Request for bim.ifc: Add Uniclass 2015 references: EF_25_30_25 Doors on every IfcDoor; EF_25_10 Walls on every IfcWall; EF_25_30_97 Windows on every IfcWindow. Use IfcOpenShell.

First a look at what the model holds.

```python
import ifcopenshell

model = ifcopenshell.open("bim.ifc")
print(model.schema)
print("classifications:", [c.Name for c in model.by_type("IfcClassification")])
for ifc_class in ("IfcDoor", "IfcRoof", "IfcStair", "IfcWall", "IfcWindow"):
    print(ifc_class, len(model.by_type(ifc_class)))
```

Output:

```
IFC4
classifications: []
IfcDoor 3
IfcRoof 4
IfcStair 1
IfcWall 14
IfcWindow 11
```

```python
import ifcopenshell
import ifcopenshell.api.classification

model = ifcopenshell.open("bim.ifc")

system = ifcopenshell.api.classification.add_classification(model, classification="Uniclass 2015")

codes = {
    "IfcDoor": ("EF_25_30_25", "Doors"),
    "IfcWall": ("EF_25_10", "Walls"),
    "IfcWindow": ("EF_25_30_97", "Windows"),
}
for ifc_class, (code, name) in codes.items():
    products = model.by_type(ifc_class)
    ifcopenshell.api.classification.add_reference(
        model, products=products, classification=system, identification=code, name=name
    )
    print(code, len(products))

model.write("bim_edited.ifc")
```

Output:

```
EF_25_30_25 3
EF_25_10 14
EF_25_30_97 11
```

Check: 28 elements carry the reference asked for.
